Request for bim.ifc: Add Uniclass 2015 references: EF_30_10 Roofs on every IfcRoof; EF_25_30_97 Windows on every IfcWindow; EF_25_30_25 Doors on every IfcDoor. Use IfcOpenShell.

First a look at what the model holds.

```python
import ifcopenshell

model = ifcopenshell.open("bim.ifc")
print(model.schema)
print("classifications:", [c.Name for c in model.by_type("IfcClassification")])
for ifc_class in ("IfcDoor", "IfcRoof", "IfcStair", "IfcWall", "IfcWindow"):
    print(ifc_class, len(model.by_type(ifc_class)))
```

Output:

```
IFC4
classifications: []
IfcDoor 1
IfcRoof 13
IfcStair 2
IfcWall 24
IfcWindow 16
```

```python
import ifcopenshell
import ifcopenshell.api.classification

model = ifcopenshell.open("bim.ifc")

system = ifcopenshell.api.classification.add_classification(model, classification="Uniclass 2015")

codes = {
    "IfcRoof": ("EF_30_10", "Roofs"),
    "IfcWindow": ("EF_25_30_97", "Windows"),
    "IfcDoor": ("EF_25_30_25", "Doors"),
}
for ifc_class, (code, name) in codes.items():
    products = model.by_type(ifc_class)
    ifcopenshell.api.classification.add_reference(
        model, products=products, classification=system, identification=code, name=name
    )
    print(code, len(products))

model.write("bim-out.ifc")
```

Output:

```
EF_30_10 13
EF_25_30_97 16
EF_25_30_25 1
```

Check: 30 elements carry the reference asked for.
